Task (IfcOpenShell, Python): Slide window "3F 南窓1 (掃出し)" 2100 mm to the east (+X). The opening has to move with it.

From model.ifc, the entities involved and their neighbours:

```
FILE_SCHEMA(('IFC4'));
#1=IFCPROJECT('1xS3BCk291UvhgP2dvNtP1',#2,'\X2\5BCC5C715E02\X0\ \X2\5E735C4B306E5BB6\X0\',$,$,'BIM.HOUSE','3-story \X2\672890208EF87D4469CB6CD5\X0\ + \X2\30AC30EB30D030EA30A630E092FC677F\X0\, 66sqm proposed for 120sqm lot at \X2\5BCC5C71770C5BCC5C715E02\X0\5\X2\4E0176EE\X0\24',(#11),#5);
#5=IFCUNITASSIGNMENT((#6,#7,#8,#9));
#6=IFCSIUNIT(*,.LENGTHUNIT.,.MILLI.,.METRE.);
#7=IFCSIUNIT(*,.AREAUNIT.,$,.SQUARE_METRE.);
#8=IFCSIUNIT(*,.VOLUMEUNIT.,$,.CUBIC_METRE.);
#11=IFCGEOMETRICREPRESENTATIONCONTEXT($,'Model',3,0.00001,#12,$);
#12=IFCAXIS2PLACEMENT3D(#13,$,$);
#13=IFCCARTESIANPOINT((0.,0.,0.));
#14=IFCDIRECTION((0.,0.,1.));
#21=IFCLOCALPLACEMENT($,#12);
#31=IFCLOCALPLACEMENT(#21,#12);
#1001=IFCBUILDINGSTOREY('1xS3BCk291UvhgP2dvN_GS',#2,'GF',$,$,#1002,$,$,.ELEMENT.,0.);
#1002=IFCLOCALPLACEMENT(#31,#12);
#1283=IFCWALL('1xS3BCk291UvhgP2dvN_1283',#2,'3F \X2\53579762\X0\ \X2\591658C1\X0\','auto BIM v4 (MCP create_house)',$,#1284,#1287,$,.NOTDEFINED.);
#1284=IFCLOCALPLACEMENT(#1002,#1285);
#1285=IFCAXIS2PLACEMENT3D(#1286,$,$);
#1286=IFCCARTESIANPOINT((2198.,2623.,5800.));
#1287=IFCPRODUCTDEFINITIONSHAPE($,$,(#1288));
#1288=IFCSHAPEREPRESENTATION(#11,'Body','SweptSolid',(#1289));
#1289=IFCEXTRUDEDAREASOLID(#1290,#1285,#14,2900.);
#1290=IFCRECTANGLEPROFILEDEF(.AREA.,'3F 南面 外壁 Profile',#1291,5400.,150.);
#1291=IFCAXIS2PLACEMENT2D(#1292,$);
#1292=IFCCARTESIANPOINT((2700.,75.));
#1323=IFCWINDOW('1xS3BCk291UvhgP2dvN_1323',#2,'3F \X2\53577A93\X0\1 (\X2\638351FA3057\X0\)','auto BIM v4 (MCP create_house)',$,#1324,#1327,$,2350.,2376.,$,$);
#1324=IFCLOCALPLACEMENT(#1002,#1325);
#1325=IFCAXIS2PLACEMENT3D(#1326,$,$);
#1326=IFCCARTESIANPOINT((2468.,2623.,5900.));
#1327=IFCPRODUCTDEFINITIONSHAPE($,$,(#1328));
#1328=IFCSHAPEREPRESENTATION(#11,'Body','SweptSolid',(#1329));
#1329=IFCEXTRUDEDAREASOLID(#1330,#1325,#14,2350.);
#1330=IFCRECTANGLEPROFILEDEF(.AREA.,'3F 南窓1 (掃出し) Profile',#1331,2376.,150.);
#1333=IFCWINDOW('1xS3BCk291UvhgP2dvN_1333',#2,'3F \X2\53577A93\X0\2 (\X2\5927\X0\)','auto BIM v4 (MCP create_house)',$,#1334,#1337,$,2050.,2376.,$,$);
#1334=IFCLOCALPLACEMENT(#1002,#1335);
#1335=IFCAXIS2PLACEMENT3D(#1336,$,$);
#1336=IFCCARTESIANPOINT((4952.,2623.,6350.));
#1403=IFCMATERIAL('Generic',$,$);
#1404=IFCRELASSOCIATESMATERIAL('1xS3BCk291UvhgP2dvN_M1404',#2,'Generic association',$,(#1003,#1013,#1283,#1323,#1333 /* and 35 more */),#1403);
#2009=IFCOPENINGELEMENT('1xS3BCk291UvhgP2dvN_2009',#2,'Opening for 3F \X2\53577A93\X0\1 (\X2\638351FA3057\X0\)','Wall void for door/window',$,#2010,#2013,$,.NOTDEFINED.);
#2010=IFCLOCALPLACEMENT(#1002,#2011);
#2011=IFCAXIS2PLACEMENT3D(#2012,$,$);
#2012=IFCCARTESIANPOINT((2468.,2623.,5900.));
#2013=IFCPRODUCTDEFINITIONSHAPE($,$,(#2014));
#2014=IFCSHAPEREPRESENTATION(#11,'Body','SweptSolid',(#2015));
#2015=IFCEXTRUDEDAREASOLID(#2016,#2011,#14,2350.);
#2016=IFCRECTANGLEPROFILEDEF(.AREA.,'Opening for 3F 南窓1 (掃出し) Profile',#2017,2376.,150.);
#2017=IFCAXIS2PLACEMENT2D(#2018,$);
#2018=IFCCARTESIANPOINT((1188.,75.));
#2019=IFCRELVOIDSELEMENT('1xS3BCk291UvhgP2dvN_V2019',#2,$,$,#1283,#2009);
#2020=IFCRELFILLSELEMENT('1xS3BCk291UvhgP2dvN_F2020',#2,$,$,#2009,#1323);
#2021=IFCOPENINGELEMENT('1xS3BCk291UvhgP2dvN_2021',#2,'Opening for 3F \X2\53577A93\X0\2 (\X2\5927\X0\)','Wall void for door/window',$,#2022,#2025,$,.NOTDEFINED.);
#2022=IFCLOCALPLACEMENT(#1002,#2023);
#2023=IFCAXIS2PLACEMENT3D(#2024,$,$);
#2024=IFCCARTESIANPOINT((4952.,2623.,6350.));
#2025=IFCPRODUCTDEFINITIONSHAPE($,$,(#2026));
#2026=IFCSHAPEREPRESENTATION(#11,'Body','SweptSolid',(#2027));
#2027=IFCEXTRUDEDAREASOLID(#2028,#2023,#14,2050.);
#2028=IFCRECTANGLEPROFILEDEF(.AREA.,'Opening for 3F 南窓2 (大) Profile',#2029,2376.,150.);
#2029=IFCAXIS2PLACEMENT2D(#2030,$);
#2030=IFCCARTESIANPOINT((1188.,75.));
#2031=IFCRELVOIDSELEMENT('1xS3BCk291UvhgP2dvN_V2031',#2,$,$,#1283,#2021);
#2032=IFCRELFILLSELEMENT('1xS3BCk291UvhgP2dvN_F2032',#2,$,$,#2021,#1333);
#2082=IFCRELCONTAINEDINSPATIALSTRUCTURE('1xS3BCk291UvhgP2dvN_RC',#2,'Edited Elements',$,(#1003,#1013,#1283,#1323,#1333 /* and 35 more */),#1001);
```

```python
import ifcopenshell
import ifcopenshell.api.geometry
import ifcopenshell.util.placement

model = ifcopenshell.open("model.ifc")

window = model.by_guid("1xS3BCk291UvhgP2dvN_1323")
opening = window.FillsVoids[0].RelatingOpeningElement
wall = opening.VoidsElements[0].RelatingBuildingElement

wall_matrix = ifcopenshell.util.placement.get_local_placement(wall.ObjectPlacement)
shift = wall_matrix[:3, 0] * 2100.0
before = ifcopenshell.util.placement.get_local_placement(window.ObjectPlacement)[:3, 3].copy()

# The window is not placed relative to its opening, so move both.
for product in (opening, window):
    matrix = ifcopenshell.util.placement.get_local_placement(product.ObjectPlacement)
    matrix[:3, 3] += shift
    ifcopenshell.api.geometry.edit_object_placement(model, product=product, matrix=matrix, is_si=False)

after = ifcopenshell.util.placement.get_local_placement(window.ObjectPlacement)[:3, 3]
print("window moved by", (after - before).round(3) + 0.0)

model.write("model_edited.ifc")
```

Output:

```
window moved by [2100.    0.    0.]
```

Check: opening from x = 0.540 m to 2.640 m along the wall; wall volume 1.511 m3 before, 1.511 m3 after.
